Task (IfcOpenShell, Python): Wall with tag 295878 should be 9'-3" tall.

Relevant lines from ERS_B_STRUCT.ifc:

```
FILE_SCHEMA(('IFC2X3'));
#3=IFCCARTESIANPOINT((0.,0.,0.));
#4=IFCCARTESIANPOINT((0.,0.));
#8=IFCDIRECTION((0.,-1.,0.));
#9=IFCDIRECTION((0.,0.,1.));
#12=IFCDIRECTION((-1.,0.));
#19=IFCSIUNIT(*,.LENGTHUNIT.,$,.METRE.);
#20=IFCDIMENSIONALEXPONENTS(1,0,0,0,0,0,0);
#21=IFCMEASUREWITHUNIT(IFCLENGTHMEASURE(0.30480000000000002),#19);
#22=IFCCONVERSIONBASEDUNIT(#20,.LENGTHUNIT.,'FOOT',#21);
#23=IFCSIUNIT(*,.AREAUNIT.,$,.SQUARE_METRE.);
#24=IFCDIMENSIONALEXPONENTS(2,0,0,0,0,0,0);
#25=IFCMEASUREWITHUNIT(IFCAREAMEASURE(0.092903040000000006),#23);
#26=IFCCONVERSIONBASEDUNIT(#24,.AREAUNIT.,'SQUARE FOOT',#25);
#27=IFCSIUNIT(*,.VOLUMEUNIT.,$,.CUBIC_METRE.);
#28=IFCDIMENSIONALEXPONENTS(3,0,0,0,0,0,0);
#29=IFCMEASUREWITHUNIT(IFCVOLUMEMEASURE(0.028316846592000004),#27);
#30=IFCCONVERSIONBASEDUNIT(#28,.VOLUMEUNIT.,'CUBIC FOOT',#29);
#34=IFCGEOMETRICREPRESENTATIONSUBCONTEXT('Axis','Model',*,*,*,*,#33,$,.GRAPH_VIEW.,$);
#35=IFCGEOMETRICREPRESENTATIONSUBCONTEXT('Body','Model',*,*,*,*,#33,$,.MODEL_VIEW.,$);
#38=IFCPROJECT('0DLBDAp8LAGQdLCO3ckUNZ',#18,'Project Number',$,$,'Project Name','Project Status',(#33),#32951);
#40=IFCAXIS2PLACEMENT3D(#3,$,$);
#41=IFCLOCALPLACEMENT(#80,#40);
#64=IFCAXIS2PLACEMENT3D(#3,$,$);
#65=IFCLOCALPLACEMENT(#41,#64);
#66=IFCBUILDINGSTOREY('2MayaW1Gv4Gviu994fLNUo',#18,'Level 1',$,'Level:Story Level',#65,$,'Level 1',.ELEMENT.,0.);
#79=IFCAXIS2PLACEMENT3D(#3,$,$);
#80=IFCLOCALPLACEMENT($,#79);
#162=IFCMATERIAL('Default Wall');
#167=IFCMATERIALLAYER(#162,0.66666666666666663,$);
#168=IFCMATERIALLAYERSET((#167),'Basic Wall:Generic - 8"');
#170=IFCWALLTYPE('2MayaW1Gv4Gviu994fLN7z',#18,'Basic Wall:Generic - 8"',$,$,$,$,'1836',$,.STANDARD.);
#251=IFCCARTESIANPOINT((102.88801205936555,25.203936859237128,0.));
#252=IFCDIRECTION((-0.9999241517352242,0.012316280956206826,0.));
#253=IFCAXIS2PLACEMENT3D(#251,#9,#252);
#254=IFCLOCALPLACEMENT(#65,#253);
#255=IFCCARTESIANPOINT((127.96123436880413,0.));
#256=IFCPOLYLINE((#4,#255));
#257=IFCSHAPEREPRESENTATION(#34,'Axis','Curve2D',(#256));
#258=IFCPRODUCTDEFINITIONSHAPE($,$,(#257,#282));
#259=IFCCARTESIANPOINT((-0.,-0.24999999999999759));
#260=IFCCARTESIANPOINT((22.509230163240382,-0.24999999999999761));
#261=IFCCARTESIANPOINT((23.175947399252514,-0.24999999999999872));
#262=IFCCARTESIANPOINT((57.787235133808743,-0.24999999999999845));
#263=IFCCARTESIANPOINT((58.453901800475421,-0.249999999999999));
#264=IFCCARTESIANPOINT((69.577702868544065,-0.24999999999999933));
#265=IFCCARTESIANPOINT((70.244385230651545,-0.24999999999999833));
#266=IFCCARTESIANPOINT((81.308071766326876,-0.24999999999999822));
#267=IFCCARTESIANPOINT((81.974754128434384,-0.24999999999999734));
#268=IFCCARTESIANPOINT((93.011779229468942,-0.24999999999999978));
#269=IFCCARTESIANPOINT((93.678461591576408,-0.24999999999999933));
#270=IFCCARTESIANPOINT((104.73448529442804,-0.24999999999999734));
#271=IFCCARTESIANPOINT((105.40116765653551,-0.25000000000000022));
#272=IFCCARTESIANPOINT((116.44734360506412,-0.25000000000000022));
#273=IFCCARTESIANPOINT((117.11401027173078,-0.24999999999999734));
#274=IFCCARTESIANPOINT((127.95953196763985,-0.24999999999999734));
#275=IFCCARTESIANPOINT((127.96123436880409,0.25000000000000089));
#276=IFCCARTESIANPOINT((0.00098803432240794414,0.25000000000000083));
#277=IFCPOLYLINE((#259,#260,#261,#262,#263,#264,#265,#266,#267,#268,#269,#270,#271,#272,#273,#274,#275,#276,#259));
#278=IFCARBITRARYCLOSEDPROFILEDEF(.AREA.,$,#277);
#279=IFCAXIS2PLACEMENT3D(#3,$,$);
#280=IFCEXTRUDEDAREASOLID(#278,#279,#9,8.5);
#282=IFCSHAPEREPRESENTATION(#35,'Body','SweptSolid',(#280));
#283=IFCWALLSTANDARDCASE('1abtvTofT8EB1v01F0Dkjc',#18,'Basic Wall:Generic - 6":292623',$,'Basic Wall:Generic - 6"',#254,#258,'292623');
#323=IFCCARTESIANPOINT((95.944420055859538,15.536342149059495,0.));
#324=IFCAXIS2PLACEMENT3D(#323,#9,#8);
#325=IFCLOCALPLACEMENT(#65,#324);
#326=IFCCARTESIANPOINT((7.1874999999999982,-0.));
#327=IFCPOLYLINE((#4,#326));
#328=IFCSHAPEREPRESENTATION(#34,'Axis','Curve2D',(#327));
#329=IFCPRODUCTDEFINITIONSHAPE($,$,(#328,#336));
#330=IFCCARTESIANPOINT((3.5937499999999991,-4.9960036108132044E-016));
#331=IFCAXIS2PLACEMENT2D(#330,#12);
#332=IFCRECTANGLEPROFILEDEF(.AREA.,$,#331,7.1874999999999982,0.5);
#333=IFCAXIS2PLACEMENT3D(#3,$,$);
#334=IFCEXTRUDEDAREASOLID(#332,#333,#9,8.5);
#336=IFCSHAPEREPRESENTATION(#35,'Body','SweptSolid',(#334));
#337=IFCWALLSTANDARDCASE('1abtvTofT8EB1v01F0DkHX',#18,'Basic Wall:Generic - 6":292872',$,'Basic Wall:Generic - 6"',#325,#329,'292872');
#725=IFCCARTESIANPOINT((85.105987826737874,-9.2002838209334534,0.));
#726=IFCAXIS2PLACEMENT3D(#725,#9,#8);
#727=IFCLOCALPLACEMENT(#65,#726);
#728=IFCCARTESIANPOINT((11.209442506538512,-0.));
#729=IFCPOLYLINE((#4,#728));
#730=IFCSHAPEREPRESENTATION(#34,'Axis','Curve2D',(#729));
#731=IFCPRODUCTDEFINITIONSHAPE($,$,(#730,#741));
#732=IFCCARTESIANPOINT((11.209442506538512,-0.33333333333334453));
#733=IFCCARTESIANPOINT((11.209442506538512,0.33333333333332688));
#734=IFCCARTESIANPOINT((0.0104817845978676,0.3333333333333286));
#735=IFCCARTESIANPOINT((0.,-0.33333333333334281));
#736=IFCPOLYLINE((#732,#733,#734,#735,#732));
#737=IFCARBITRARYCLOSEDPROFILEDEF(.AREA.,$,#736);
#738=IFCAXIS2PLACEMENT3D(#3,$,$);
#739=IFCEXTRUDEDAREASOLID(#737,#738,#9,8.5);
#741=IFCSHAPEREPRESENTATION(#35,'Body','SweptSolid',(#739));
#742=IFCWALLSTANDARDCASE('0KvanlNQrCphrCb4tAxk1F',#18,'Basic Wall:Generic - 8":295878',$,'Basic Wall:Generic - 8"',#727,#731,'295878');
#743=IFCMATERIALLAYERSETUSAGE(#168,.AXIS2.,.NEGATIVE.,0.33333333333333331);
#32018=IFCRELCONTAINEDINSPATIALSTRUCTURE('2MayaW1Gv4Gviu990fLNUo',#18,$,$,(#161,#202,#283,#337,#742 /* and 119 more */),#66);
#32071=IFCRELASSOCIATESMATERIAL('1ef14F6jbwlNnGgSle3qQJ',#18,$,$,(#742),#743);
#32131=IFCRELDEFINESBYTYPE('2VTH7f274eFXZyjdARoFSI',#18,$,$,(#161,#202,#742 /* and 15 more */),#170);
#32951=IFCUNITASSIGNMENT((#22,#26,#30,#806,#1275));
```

```python
import ifcopenshell
import ifcopenshell.geom
import ifcopenshell.util.representation
import ifcopenshell.util.shape
import ifcopenshell.util.unit

model = ifcopenshell.open("ERS_B_STRUCT.ifc")
unit_scale = ifcopenshell.util.unit.calculate_unit_scale(model)
settings = ifcopenshell.geom.settings()


def volume(element):
    """Net volume in cubic metres, openings subtracted."""
    shape = ifcopenshell.geom.create_shape(settings, element)
    return ifcopenshell.util.shape.get_volume(shape.geometry)


wall = model.by_guid("0KvanlNQrCphrCb4tAxk1F")
before = volume(wall)

body = ifcopenshell.util.representation.get_representation(wall, "Model", "Body")
solid = body.Items[0]
old_height = solid.Depth
solid.Depth = 111 * 0.0254 / unit_scale
after = volume(wall)

print(f"height {old_height:g} -> {solid.Depth:g}, volume {before:.3f} -> {after:.3f} m3")

model.write("ERS_B_STRUCT_updated.ifc")
```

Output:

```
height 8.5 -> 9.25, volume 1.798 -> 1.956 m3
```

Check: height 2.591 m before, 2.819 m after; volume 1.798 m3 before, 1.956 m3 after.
